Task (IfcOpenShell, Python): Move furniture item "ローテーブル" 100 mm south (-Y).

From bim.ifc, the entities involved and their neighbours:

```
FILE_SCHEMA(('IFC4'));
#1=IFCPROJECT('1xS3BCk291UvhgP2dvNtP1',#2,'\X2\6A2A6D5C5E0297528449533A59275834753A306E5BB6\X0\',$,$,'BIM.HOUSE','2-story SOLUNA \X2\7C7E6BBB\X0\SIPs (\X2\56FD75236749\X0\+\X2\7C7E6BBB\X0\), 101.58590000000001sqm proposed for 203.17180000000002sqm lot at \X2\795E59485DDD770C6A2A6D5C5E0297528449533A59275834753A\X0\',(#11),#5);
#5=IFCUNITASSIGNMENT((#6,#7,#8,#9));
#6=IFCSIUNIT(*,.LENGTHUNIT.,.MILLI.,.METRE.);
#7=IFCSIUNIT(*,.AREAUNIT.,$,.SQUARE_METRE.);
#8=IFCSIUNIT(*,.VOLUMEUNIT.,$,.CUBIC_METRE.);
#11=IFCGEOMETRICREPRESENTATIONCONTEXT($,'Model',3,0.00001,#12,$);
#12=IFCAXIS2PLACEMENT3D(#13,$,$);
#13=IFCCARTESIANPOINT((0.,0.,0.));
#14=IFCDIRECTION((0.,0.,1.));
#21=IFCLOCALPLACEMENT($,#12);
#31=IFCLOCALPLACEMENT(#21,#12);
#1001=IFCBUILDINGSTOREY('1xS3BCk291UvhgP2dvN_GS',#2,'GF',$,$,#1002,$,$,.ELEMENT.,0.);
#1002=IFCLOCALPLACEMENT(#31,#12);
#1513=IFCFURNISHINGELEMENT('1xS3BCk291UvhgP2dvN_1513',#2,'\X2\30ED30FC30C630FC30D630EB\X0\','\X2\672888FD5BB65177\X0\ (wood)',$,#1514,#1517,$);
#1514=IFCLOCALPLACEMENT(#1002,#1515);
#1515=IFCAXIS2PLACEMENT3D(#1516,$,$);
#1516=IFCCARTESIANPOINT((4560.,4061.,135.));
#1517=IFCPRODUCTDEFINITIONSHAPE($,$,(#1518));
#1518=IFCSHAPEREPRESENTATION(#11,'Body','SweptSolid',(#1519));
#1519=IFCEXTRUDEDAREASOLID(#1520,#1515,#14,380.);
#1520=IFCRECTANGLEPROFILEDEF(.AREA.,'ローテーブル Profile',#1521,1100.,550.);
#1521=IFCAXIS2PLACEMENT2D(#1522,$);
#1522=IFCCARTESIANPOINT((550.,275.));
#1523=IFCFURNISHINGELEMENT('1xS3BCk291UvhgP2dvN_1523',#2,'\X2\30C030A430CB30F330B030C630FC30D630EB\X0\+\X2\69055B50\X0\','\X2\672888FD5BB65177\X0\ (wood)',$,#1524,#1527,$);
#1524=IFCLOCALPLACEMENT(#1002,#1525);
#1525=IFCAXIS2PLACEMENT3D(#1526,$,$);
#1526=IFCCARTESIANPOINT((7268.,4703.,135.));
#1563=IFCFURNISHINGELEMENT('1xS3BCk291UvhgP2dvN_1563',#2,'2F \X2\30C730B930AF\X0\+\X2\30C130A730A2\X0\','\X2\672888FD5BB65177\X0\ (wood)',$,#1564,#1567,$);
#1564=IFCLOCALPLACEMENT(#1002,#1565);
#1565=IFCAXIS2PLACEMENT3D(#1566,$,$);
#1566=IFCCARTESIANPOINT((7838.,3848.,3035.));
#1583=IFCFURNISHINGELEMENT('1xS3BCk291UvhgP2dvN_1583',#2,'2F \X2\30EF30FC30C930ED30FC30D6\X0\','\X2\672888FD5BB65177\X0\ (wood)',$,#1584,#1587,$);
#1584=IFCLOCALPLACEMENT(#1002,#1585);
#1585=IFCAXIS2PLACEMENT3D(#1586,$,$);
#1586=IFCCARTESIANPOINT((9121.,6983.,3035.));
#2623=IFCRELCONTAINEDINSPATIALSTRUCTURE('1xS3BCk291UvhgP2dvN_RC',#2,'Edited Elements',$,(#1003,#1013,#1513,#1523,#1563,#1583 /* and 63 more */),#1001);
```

```python
import ifcopenshell
import ifcopenshell.api.geometry
import ifcopenshell.util.placement

model = ifcopenshell.open("bim.ifc")

item = model.by_guid("1xS3BCk291UvhgP2dvN_1513")
matrix = ifcopenshell.util.placement.get_local_placement(item.ObjectPlacement)
matrix[1, 3] -= 100.0
ifcopenshell.api.geometry.edit_object_placement(model, product=item, matrix=matrix, is_si=False)

print(ifcopenshell.util.placement.get_local_placement(item.ObjectPlacement).round(3) + 0.0)

model.write("bim-out.ifc")
```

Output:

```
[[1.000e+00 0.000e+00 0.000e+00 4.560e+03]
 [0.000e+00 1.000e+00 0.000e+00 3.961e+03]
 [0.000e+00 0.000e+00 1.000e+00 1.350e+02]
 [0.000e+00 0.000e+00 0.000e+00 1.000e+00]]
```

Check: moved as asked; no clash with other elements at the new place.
